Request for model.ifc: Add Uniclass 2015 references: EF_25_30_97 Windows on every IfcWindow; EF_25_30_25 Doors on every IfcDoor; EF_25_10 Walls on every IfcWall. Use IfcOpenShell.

First a look at what the model holds.

```python
import ifcopenshell

model = ifcopenshell.open("model.ifc")
print(model.schema)
print("classifications:", [c.Name for c in model.by_type("IfcClassification")])
for ifc_class in ("IfcDoor", "IfcRoof", "IfcStair", "IfcWall", "IfcWindow"):
    print(ifc_class, len(model.by_type(ifc_class)))
```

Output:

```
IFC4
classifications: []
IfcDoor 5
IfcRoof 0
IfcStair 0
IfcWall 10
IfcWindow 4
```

```python
import ifcopenshell
import ifcopenshell.api.classification

model = ifcopenshell.open("model.ifc")

system = ifcopenshell.api.classification.add_classification(model, classification="Uniclass 2015")

codes = {
    "IfcWindow": ("EF_25_30_97", "Windows"),
    "IfcDoor": ("EF_25_30_25", "Doors"),
    "IfcWall": ("EF_25_10", "Walls"),
}
for ifc_class, (code, name) in codes.items():
    products = model.by_type(ifc_class)
    ifcopenshell.api.classification.add_reference(
        model, products=products, classification=system, identification=code, name=name
    )
    print(code, len(products))

model.write("model-out.ifc")
```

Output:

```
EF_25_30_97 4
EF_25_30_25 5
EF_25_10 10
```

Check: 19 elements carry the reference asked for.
